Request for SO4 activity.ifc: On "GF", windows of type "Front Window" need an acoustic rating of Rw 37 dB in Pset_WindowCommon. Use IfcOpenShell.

First a look at what the model holds.

```python
import ifcopenshell
import ifcopenshell.util.element

model = ifcopenshell.open("SO4 activity.ifc")
print(model.schema)
storey = next(s for s in model.by_type("IfcBuildingStorey") if s.Name == "GF")
windows = [e for e in ifcopenshell.util.element.get_decomposition(storey) if e.is_a("IfcWindow")]
seen = {}
for e in windows:
    element_type = ifcopenshell.util.element.get_type(e)
    key = (element_type.Name if element_type != e and element_type else None, ifcopenshell.util.element.get_pset(e, "Pset_WindowCommon", "AcousticRating"))
    seen[key] = seen.get(key, 0) + 1
for (name, value), count in sorted(seen.items(), key=str):
    print(count, "x", name, "|", value)
```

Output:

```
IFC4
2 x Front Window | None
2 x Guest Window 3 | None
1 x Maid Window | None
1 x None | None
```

```python
import ifcopenshell
import ifcopenshell.api.pset
import ifcopenshell.util.element

model = ifcopenshell.open("SO4 activity.ifc")

storey = next(s for s in model.by_type("IfcBuildingStorey") if s.Name == "GF")
windows = [e for e in ifcopenshell.util.element.get_decomposition(storey) if e.is_a("IfcWindow")]

count = 0
for e in windows:
    element_type = ifcopenshell.util.element.get_type(e)
    if element_type in (None, e) or element_type.Name != "Front Window":
        continue
    # add_pset returns the element's existing set when there is one.
    pset = ifcopenshell.api.pset.add_pset(model, product=e, name="Pset_WindowCommon")
    ifcopenshell.api.pset.edit_pset(model, pset=pset, properties={"AcousticRating": "Rw 37 dB"})
    count += 1

print(count, "windows updated")

model.write("SO4 activity_updated.ifc")
```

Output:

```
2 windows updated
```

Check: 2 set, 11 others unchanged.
